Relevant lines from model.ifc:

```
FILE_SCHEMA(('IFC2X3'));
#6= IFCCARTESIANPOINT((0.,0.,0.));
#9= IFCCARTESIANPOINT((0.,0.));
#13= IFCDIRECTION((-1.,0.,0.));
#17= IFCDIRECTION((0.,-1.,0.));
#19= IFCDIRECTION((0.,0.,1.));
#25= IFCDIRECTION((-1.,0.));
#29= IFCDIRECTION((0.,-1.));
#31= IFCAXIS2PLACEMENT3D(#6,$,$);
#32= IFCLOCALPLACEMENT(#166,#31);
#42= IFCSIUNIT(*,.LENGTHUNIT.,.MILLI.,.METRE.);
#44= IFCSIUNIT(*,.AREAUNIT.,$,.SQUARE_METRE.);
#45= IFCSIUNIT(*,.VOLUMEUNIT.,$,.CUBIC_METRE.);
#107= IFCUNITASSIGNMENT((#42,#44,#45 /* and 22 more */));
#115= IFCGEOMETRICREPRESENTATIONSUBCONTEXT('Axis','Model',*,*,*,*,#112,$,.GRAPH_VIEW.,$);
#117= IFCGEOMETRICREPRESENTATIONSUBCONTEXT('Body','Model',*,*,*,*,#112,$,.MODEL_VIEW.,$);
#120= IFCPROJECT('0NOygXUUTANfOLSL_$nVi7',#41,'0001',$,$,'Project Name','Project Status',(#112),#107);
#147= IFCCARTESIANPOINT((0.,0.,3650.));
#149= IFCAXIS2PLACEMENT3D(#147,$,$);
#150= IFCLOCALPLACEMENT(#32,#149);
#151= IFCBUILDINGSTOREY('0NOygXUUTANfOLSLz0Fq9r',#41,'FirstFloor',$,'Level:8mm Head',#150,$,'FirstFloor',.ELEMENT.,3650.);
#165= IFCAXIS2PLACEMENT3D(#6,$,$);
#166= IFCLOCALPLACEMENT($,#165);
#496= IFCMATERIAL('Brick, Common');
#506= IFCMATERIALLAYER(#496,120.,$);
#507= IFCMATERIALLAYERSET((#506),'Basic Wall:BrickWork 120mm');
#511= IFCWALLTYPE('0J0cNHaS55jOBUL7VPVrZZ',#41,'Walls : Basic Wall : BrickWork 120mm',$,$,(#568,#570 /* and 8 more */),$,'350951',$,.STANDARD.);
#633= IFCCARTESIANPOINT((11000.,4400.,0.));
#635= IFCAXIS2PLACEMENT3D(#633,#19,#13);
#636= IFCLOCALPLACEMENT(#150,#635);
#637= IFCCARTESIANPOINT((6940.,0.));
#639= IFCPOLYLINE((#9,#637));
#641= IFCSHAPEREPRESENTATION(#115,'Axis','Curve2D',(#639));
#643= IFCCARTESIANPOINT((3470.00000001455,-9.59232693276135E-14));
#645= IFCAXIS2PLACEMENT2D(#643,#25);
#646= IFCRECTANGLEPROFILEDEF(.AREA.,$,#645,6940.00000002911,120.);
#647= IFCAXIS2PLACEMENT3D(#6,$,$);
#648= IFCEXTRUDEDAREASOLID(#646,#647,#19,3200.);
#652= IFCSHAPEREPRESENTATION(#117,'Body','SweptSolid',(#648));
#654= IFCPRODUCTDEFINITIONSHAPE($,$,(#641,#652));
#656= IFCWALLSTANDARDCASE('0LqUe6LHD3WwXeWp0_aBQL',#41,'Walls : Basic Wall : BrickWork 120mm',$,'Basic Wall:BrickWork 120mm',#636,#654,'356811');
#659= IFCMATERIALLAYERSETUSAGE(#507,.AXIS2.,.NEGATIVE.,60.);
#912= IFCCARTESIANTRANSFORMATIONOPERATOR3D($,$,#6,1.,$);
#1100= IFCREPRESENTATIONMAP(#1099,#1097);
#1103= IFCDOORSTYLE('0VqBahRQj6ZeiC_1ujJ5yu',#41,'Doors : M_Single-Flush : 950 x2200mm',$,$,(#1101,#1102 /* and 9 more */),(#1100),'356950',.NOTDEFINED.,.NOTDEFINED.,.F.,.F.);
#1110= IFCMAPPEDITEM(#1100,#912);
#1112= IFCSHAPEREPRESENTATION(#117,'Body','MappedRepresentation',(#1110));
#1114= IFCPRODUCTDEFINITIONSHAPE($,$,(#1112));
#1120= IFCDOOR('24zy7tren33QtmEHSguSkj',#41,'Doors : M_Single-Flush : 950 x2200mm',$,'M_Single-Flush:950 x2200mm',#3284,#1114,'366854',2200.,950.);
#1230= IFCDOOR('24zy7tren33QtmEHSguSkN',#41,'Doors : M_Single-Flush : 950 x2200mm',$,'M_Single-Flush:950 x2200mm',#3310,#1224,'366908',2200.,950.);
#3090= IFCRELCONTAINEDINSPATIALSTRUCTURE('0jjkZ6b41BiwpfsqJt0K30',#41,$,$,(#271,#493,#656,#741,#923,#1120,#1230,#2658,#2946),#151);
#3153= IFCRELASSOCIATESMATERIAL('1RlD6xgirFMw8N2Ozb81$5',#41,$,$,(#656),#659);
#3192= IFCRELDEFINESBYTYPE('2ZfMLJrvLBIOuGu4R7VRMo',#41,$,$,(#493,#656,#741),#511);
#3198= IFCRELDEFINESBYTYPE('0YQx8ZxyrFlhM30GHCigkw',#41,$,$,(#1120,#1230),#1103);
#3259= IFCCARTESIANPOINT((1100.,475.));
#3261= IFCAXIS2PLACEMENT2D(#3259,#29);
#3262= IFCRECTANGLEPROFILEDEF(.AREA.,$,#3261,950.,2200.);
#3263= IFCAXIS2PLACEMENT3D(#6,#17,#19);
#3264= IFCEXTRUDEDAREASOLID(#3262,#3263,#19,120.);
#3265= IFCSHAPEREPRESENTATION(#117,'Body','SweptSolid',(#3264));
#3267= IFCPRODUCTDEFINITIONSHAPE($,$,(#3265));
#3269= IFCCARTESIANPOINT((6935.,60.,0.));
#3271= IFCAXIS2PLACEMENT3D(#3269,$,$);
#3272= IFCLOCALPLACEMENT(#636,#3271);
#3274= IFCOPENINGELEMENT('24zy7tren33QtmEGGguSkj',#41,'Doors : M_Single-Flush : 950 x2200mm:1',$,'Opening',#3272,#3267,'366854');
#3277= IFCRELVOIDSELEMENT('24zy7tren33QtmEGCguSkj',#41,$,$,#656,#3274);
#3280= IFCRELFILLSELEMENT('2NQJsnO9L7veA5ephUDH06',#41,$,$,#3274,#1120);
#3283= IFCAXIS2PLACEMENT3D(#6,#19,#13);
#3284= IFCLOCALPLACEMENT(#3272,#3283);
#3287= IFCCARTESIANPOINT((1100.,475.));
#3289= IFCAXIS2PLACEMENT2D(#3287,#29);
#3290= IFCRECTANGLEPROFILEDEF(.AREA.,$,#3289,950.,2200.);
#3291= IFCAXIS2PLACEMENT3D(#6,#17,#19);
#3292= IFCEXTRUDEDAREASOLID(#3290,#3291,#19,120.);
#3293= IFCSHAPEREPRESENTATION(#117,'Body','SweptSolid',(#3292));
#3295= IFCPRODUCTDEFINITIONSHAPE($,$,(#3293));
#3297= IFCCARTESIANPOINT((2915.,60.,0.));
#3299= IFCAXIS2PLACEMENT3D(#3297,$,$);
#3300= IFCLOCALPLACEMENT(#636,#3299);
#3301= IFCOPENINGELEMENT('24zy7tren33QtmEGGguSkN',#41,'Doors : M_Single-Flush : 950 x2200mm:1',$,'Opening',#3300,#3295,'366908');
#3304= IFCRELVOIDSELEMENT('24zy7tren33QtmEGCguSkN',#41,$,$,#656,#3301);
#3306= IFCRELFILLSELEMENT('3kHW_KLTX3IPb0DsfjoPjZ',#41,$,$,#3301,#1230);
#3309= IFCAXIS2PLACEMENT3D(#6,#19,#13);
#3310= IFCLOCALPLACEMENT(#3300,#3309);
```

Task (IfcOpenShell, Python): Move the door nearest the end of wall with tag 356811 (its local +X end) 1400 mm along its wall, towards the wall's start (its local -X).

```python
import ifcopenshell
import ifcopenshell.api.geometry
import ifcopenshell.util.placement
import ifcopenshell.util.unit

model = ifcopenshell.open("model.ifc")
unit_scale = ifcopenshell.util.unit.calculate_unit_scale(model)

door = model.by_guid("24zy7tren33QtmEHSguSkj")
opening = door.FillsVoids[0].RelatingOpeningElement
wall = opening.VoidsElements[0].RelatingBuildingElement

wall_matrix = ifcopenshell.util.placement.get_local_placement(wall.ObjectPlacement)
shift = wall_matrix[:3, 0] * -1.4 / unit_scale
before = ifcopenshell.util.placement.get_local_placement(door.ObjectPlacement)[:3, 3].copy()

# The door is placed relative to its opening, so it follows when the opening moves.
matrix = ifcopenshell.util.placement.get_local_placement(opening.ObjectPlacement)
matrix[:3, 3] += shift
ifcopenshell.api.geometry.edit_object_placement(
    model, product=opening, matrix=matrix, is_si=False, should_transform_children=True
)

after = ifcopenshell.util.placement.get_local_placement(door.ObjectPlacement)[:3, 3]
print("door moved by", (after - before).round(3) + 0.0)

model.write("model_v2.ifc")
```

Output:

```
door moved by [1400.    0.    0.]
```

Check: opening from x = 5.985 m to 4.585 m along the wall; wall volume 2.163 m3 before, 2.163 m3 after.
